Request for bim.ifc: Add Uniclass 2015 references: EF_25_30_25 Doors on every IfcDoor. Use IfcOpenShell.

First a look at what the model holds.

```python
import ifcopenshell

model = ifcopenshell.open("bim.ifc")
print(model.schema)
print("classifications:", [c.Name for c in model.by_type("IfcClassification")])
for ifc_class in ("IfcDoor", "IfcRoof", "IfcStair", "IfcWall", "IfcWindow"):
    print(ifc_class, len(model.by_type(ifc_class)))
```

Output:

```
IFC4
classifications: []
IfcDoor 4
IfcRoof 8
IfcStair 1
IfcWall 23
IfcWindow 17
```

```python
import ifcopenshell
import ifcopenshell.api.classification

model = ifcopenshell.open("bim.ifc")

system = ifcopenshell.api.classification.add_classification(model, classification="Uniclass 2015")

codes = {
    "IfcDoor": ("EF_25_30_25", "Doors"),
}
for ifc_class, (code, name) in codes.items():
    products = model.by_type(ifc_class)
    ifcopenshell.api.classification.add_reference(
        model, products=products, classification=system, identification=code, name=name
    )
    print(code, len(products))

model.write("bim_v2.ifc")
```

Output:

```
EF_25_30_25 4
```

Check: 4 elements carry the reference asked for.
